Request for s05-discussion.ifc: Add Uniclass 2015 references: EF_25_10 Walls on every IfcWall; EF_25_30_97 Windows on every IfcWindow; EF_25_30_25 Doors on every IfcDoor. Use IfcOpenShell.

First a look at what the model holds.

```python
import ifcopenshell

model = ifcopenshell.open("s05-discussion.ifc")
print(model.schema)
print("classifications:", [c.Name for c in model.by_type("IfcClassification")])
for ifc_class in ("IfcDoor", "IfcRoof", "IfcStair", "IfcWall", "IfcWindow"):
    print(ifc_class, len(model.by_type(ifc_class)))
```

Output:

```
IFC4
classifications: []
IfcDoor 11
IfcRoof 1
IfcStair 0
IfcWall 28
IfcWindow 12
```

```python
import ifcopenshell
import ifcopenshell.api.classification

model = ifcopenshell.open("s05-discussion.ifc")

system = ifcopenshell.api.classification.add_classification(model, classification="Uniclass 2015")

codes = {
    "IfcWall": ("EF_25_10", "Walls"),
    "IfcWindow": ("EF_25_30_97", "Windows"),
    "IfcDoor": ("EF_25_30_25", "Doors"),
}
for ifc_class, (code, name) in codes.items():
    products = model.by_type(ifc_class)
    ifcopenshell.api.classification.add_reference(
        model, products=products, classification=system, identification=code, name=name
    )
    print(code, len(products))

model.write("s05-discussion-out.ifc")
```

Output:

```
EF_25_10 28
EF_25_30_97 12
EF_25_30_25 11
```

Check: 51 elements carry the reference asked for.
